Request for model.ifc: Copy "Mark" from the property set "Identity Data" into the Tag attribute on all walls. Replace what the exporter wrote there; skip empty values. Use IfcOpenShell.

First a look at what the model holds.

```python
import ifcopenshell
import ifcopenshell.util.element

model = ifcopenshell.open("model.ifc")
print(model.schema)
walls = model.by_type("IfcWall")
print(len(walls), "walls")
for e in walls[:8]:
    source = ifcopenshell.util.element.get_pset(e, "Identity Data", "Mark")
    target = e.Tag
    print(e.id(), repr(source), repr(target), sep=" | ")
```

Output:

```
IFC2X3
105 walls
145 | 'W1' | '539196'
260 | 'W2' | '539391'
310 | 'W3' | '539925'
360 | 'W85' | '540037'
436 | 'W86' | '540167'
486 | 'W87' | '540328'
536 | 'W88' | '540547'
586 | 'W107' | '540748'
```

```python
import ifcopenshell
import ifcopenshell.util.element

model = ifcopenshell.open("model.ifc")

count = 0
for e in model.by_type("IfcWall"):
    value = ifcopenshell.util.element.get_pset(e, "Identity Data", "Mark")
    current = e.Tag
    if not value or not value.strip() or current == value:
        continue
    e.Tag = value
    count += 1

print(count, "walls updated")

model.write("model_updated.ifc")
```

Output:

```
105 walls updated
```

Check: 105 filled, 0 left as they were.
